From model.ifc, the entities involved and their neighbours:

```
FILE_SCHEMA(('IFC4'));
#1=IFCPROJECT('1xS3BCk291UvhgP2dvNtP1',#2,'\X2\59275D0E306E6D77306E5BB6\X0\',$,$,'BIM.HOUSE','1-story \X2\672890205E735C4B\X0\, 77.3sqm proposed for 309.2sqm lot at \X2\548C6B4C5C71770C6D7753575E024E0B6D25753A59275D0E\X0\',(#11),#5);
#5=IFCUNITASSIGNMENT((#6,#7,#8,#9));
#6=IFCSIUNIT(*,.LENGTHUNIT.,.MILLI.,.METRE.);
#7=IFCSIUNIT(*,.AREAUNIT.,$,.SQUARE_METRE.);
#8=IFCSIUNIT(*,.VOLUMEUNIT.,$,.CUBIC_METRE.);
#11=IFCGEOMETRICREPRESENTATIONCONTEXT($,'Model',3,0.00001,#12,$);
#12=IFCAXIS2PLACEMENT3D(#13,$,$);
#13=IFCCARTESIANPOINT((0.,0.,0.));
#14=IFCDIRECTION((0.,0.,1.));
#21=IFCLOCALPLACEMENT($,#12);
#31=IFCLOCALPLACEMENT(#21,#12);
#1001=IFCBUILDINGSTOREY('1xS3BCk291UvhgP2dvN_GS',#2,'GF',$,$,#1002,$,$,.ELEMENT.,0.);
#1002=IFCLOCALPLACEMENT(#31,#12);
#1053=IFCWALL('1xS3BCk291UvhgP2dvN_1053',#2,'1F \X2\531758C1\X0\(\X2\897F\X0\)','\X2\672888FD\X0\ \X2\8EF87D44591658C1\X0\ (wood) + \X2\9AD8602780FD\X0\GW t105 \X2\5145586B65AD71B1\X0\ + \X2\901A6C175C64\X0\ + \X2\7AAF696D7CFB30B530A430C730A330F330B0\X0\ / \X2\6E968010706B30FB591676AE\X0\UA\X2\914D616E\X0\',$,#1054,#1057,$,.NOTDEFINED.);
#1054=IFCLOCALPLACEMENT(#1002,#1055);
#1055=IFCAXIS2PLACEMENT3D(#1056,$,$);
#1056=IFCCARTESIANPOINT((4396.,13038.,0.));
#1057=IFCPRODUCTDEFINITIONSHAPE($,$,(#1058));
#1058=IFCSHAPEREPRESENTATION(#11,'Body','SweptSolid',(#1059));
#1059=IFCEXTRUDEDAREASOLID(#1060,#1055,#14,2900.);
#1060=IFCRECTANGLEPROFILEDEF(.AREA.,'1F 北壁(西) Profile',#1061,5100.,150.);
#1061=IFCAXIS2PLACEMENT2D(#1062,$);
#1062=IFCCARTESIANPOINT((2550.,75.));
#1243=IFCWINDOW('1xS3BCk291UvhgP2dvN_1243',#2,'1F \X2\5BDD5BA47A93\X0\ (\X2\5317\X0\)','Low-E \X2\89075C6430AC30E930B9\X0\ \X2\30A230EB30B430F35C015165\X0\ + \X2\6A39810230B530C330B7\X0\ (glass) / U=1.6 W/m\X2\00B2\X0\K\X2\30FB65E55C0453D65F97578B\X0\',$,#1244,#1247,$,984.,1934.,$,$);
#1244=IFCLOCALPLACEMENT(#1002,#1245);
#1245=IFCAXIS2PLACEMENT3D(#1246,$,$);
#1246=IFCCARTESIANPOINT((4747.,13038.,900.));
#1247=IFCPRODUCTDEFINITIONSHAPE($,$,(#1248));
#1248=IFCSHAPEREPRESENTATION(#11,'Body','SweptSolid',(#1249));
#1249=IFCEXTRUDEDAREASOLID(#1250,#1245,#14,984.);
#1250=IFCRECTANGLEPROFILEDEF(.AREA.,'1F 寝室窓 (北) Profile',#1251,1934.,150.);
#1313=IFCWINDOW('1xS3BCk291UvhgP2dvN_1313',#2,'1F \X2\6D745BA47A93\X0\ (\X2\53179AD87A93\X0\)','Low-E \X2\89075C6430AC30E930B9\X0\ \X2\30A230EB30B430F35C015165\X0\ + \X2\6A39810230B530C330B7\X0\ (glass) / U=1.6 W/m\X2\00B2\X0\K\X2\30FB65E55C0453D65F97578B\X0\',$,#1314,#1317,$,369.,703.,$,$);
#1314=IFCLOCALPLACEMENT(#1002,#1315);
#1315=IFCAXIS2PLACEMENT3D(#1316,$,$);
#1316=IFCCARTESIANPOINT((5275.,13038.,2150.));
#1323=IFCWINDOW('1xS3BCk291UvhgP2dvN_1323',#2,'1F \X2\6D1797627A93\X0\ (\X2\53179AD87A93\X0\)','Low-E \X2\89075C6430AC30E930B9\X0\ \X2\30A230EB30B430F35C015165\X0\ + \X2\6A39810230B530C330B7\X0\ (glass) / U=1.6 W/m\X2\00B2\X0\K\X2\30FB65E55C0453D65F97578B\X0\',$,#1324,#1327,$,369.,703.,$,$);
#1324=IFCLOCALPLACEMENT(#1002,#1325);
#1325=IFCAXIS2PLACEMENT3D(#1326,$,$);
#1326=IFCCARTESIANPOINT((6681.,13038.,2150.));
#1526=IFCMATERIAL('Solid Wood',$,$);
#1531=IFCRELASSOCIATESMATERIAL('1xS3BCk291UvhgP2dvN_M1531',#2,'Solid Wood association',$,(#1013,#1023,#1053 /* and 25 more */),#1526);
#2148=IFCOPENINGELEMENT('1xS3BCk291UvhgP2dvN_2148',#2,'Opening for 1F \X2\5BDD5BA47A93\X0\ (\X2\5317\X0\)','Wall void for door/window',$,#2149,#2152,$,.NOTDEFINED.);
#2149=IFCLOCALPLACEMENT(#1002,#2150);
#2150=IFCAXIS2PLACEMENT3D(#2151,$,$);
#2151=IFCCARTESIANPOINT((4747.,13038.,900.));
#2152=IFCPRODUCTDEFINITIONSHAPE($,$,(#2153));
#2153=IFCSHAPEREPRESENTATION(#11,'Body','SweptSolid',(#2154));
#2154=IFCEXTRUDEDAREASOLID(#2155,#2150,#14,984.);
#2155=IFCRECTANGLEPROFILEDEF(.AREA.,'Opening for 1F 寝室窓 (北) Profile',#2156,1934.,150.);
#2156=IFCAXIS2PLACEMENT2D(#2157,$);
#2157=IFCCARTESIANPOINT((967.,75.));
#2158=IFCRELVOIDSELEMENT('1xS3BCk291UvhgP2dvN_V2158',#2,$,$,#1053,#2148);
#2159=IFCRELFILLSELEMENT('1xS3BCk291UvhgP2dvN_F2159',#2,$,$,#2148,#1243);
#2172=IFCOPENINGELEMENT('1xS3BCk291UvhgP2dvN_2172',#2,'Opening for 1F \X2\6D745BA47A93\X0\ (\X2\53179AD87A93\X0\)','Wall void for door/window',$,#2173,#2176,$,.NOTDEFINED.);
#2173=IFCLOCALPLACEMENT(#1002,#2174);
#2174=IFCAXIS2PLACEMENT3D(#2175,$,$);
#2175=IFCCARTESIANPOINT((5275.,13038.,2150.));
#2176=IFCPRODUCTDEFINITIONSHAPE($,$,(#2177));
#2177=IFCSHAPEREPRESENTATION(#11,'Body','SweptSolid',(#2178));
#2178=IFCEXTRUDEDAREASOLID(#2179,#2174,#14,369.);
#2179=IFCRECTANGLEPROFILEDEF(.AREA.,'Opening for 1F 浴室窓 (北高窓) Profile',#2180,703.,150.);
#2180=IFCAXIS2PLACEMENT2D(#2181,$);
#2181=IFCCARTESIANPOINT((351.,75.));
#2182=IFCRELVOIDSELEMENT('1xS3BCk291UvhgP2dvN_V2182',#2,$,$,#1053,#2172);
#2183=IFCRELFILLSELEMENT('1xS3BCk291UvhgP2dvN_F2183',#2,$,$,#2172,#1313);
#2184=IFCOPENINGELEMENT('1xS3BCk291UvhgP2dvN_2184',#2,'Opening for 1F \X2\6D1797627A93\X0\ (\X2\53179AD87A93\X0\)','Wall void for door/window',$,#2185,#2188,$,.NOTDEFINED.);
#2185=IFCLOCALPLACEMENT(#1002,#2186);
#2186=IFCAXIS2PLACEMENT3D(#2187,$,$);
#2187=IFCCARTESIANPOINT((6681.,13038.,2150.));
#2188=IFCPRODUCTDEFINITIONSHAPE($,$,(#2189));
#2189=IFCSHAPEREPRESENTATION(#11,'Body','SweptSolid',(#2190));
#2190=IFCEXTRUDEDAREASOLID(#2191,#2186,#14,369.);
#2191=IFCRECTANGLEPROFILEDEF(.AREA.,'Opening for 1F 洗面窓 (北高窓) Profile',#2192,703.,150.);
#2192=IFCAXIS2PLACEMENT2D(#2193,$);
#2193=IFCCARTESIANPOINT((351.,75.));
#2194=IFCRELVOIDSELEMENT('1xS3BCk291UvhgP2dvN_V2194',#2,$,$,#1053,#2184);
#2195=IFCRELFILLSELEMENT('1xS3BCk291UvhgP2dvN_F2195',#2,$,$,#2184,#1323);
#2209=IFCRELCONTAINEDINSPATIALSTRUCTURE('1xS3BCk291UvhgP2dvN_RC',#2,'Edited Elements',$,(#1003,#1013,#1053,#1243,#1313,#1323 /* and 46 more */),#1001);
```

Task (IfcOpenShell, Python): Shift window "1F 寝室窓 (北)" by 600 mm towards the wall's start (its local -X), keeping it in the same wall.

```python
import ifcopenshell
import ifcopenshell.api.geometry
import ifcopenshell.util.placement
import ifcopenshell.util.unit

model = ifcopenshell.open("model.ifc")
unit_scale = ifcopenshell.util.unit.calculate_unit_scale(model)

window = model.by_guid("1xS3BCk291UvhgP2dvN_1243")
opening = window.FillsVoids[0].RelatingOpeningElement
wall = opening.VoidsElements[0].RelatingBuildingElement

wall_matrix = ifcopenshell.util.placement.get_local_placement(wall.ObjectPlacement)
shift = wall_matrix[:3, 0] * -0.6 / unit_scale
before = ifcopenshell.util.placement.get_local_placement(window.ObjectPlacement)[:3, 3].copy()

# The window is not placed relative to its opening, so move both.
for product in (opening, window):
    matrix = ifcopenshell.util.placement.get_local_placement(product.ObjectPlacement)
    matrix[:3, 3] += shift
    ifcopenshell.api.geometry.edit_object_placement(model, product=product, matrix=matrix, is_si=False)

after = ifcopenshell.util.placement.get_local_placement(window.ObjectPlacement)[:3, 3]
print("window moved by", (after - before).round(3) + 0.0)

model.write("model_edited.ifc")
```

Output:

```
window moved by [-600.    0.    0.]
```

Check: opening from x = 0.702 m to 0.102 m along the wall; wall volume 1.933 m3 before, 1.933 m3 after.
